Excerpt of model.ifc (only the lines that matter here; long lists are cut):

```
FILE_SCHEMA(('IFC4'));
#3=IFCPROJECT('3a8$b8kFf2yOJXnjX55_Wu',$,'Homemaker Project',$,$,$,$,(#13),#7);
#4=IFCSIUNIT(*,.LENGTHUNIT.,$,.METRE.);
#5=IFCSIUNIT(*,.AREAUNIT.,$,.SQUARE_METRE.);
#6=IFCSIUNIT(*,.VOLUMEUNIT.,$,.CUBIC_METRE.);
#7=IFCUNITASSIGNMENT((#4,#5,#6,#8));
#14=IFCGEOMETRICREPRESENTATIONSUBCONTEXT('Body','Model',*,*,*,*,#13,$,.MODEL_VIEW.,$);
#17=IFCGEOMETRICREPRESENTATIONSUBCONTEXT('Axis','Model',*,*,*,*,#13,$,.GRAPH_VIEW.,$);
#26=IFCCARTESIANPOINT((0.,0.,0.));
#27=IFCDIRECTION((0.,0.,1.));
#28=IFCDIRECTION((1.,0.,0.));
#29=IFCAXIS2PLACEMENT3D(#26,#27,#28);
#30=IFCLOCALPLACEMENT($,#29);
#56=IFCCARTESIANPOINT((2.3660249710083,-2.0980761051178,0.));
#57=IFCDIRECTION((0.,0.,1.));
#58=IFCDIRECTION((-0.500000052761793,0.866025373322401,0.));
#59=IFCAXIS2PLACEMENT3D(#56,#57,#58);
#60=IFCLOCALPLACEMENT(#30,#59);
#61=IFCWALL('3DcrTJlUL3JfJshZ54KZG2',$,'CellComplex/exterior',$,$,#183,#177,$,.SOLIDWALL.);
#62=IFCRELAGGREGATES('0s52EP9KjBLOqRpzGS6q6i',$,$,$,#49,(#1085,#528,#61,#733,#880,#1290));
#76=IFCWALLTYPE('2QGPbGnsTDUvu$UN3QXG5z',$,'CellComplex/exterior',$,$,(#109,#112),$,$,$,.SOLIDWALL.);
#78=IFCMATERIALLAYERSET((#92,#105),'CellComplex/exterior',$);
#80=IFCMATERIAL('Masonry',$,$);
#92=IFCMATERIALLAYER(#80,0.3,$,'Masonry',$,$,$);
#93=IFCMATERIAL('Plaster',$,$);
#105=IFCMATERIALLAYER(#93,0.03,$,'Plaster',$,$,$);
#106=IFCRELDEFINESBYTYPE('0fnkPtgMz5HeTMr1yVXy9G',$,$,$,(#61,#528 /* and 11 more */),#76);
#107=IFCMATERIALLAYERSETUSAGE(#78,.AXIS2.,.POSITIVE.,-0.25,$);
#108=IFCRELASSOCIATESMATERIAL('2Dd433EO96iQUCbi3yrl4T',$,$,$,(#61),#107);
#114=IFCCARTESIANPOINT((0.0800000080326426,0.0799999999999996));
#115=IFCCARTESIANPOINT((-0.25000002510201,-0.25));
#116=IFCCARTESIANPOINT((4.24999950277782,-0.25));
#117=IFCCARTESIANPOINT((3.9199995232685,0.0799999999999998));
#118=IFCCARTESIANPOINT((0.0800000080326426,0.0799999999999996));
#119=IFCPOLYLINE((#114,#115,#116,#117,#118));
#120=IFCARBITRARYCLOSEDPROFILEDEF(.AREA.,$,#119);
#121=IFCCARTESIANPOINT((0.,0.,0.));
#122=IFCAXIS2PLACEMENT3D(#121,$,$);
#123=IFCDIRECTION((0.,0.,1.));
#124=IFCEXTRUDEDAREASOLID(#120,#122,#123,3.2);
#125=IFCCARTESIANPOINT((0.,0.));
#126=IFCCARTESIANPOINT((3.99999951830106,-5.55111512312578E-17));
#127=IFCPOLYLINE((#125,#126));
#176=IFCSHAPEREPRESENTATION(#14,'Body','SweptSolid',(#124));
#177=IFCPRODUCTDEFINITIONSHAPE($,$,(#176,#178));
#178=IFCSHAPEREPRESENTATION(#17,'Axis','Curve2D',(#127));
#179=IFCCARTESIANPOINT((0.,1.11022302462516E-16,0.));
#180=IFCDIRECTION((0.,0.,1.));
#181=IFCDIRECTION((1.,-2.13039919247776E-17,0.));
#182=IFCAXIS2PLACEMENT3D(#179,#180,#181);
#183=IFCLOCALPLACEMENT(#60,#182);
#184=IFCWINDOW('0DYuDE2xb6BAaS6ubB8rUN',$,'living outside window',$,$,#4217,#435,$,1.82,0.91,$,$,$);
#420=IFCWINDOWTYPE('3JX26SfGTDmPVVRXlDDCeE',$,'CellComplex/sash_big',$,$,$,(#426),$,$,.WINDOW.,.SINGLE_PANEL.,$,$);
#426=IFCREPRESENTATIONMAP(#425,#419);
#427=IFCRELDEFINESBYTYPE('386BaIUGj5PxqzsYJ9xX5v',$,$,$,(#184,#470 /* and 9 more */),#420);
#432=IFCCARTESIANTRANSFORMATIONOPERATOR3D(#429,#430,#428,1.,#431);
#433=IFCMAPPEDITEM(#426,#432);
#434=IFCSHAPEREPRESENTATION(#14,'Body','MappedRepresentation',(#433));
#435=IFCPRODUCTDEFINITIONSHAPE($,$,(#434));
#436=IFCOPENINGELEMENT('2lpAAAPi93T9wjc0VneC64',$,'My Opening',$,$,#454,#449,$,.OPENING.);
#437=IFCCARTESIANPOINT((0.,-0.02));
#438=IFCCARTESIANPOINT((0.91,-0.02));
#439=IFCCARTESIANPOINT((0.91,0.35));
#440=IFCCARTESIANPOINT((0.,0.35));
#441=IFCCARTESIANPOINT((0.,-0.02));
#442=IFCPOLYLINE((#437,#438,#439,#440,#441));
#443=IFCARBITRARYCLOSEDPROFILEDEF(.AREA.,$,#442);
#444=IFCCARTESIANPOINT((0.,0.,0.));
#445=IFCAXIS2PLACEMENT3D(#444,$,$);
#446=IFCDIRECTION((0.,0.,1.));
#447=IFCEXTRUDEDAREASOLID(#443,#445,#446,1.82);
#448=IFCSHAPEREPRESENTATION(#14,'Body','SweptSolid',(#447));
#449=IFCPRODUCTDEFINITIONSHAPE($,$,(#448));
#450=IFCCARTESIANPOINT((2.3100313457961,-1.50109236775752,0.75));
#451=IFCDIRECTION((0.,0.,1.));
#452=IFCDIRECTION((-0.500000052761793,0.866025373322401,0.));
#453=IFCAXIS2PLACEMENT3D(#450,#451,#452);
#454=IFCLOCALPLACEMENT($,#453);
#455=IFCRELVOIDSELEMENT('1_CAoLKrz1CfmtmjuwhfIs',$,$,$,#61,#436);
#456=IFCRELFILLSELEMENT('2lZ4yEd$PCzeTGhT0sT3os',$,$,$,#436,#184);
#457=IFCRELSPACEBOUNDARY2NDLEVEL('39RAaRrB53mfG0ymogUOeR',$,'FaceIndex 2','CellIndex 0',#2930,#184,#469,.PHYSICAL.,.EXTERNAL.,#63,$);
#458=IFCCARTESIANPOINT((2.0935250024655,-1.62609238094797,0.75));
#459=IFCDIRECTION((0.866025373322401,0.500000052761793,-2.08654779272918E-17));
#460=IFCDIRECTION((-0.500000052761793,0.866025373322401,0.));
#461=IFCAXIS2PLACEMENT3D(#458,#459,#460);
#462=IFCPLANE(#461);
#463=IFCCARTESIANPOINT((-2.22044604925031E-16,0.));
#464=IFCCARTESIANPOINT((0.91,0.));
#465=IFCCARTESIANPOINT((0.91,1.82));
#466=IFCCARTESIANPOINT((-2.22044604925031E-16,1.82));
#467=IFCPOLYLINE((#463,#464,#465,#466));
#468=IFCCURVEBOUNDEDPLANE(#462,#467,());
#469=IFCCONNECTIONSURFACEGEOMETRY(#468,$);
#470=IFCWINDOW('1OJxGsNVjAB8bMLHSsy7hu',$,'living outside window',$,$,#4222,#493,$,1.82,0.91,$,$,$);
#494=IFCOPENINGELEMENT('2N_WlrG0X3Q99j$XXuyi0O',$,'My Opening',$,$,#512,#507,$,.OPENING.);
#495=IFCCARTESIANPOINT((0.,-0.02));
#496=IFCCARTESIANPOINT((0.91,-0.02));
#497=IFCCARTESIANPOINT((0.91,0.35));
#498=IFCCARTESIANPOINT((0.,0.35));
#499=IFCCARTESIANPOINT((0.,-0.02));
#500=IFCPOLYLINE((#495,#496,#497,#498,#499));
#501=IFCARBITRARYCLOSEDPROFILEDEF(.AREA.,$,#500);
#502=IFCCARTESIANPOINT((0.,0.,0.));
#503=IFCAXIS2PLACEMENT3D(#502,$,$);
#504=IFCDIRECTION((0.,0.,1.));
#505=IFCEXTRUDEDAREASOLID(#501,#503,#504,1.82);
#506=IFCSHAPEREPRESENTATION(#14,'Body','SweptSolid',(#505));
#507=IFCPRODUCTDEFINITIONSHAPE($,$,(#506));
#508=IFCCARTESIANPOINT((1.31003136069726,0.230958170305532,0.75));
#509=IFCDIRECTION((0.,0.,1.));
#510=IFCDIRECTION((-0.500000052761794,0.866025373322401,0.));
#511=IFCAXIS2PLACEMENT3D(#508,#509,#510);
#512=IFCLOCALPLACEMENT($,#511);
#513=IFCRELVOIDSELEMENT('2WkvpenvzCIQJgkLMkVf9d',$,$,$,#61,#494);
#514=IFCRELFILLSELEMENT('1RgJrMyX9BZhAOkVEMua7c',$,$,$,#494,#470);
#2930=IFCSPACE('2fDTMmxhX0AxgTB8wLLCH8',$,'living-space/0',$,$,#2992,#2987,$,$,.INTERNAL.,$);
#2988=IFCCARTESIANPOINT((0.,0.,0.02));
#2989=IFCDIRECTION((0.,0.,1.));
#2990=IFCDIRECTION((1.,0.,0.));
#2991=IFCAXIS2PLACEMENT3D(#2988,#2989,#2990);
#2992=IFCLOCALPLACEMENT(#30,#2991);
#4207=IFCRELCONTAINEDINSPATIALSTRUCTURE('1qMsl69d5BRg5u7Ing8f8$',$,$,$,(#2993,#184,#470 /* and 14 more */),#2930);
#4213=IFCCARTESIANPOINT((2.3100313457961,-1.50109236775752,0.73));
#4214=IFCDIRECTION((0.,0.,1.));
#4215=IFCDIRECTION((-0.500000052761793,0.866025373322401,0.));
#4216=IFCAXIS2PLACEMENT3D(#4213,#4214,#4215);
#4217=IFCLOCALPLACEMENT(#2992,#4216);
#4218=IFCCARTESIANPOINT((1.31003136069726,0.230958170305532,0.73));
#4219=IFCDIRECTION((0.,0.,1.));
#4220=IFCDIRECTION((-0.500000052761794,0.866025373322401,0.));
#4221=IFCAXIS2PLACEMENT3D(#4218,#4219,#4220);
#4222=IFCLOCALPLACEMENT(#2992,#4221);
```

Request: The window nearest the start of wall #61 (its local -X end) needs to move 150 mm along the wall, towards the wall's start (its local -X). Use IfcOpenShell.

```python
import numpy as np
import ifcopenshell
import ifcopenshell.api.geometry
import ifcopenshell.util.placement
import ifcopenshell.util.unit

model = ifcopenshell.open("model.ifc")
unit_scale = ifcopenshell.util.unit.calculate_unit_scale(model)

window = model.by_guid("0DYuDE2xb6BAaS6ubB8rUN")
opening = window.FillsVoids[0].RelatingOpeningElement
wall = opening.VoidsElements[0].RelatingBuildingElement

wall_matrix = ifcopenshell.util.placement.get_local_placement(wall.ObjectPlacement)
shift = wall_matrix[:3, 0] * -0.15 / unit_scale
before = ifcopenshell.util.placement.get_local_placement(window.ObjectPlacement)[:3, 3].copy()

# The window is not placed relative to its opening, so move both.
for product in (opening, window):
    matrix = ifcopenshell.util.placement.get_local_placement(product.ObjectPlacement)
    matrix[:3, 3] += shift
    ifcopenshell.api.geometry.edit_object_placement(model, product=product, matrix=matrix, is_si=False)

# Space boundary surfaces are stored in each space's coordinates; move them too.
for rel in window.ProvidesBoundaries:
    if not rel.ConnectionGeometry:
        continue
    surface = rel.ConnectionGeometry.SurfaceOnRelatingElement.BasisSurface
    space_matrix = ifcopenshell.util.placement.get_local_placement(rel.RelatingSpace.ObjectPlacement)
    point = np.array(surface.Position.Location.Coordinates) + space_matrix[:3, :3].T @ shift
    surface.Position = model.createIfcAxis2Placement3D(
        model.createIfcCartesianPoint(point.tolist()), surface.Position.Axis, surface.Position.RefDirection
    )

after = ifcopenshell.util.placement.get_local_placement(window.ObjectPlacement)[:3, 3]
print("window moved by", (after - before).round(3) + 0.0)

model.write("model_rev.ifc")
```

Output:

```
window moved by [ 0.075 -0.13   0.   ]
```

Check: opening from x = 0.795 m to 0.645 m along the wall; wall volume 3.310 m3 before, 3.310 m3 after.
